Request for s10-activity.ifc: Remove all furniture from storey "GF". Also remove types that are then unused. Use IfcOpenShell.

First a look at what the model holds.

```python
import ifcopenshell
import ifcopenshell.util.element

model = ifcopenshell.open("s10-activity.ifc")
print(model.schema)
storey = next(s for s in model.by_type("IfcBuildingStorey") if s.Name == "GF")
furniture = [e for e in ifcopenshell.util.element.get_decomposition(storey) if e.is_a("IfcFurnishingElement")]
seen = {}
for e in furniture:
    element_type = ifcopenshell.util.element.get_type(e)
    name = element_type.Name if element_type not in (None, e) else None
    seen[name] = seen.get(name, 0) + 1
for name, count in sorted(seen.items(), key=str):
    print(count, "x", name)
```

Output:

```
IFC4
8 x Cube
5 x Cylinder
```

```python
import ifcopenshell
import ifcopenshell.api.root
import ifcopenshell.util.element

model = ifcopenshell.open("s10-activity.ifc")

storey = next(s for s in model.by_type("IfcBuildingStorey") if s.Name == "GF")
furniture = [e for e in ifcopenshell.util.element.get_decomposition(storey) if e.is_a("IfcFurnishingElement")]
types = {ifcopenshell.util.element.get_type(e) for e in furniture} - {None, *furniture}

for e in furniture:
    ifcopenshell.api.root.remove_product(model, product=e)
print(len(furniture), "removed")

unused = [t for t in types if not ifcopenshell.util.element.get_types(t)]
for t in unused:
    ifcopenshell.api.root.remove_product(model, product=t)
print(len(unused), "unused types removed")

model.write("s10-activity_v2.ifc")
```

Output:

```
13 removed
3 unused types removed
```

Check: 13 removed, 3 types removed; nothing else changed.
